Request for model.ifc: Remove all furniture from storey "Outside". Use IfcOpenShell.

First a look at what the model holds.

```python
import ifcopenshell
import ifcopenshell.util.element

model = ifcopenshell.open("model.ifc")
print(model.schema)
storey = next(s for s in model.by_type("IfcBuildingStorey") if s.Name == "Outside")
furniture = [e for e in ifcopenshell.util.element.get_decomposition(storey) if e.is_a("IfcFurnishingElement")]
seen = {}
for e in furniture:
    element_type = ifcopenshell.util.element.get_type(e)
    name = element_type.Name if element_type not in (None, e) else None
    seen[name] = seen.get(name, 0) + 1
for name, count in sorted(seen.items(), key=str):
    print(count, "x", name)
```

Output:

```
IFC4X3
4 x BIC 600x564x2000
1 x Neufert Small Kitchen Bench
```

```python
import ifcopenshell
import ifcopenshell.api.root
import ifcopenshell.util.element

model = ifcopenshell.open("model.ifc")

storey = next(s for s in model.by_type("IfcBuildingStorey") if s.Name == "Outside")
furniture = [e for e in ifcopenshell.util.element.get_decomposition(storey) if e.is_a("IfcFurnishingElement")]

for e in furniture:
    ifcopenshell.api.root.remove_product(model, product=e)
print(len(furniture), "removed")

model.write("model_v2.ifc")
```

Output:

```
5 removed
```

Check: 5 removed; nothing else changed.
